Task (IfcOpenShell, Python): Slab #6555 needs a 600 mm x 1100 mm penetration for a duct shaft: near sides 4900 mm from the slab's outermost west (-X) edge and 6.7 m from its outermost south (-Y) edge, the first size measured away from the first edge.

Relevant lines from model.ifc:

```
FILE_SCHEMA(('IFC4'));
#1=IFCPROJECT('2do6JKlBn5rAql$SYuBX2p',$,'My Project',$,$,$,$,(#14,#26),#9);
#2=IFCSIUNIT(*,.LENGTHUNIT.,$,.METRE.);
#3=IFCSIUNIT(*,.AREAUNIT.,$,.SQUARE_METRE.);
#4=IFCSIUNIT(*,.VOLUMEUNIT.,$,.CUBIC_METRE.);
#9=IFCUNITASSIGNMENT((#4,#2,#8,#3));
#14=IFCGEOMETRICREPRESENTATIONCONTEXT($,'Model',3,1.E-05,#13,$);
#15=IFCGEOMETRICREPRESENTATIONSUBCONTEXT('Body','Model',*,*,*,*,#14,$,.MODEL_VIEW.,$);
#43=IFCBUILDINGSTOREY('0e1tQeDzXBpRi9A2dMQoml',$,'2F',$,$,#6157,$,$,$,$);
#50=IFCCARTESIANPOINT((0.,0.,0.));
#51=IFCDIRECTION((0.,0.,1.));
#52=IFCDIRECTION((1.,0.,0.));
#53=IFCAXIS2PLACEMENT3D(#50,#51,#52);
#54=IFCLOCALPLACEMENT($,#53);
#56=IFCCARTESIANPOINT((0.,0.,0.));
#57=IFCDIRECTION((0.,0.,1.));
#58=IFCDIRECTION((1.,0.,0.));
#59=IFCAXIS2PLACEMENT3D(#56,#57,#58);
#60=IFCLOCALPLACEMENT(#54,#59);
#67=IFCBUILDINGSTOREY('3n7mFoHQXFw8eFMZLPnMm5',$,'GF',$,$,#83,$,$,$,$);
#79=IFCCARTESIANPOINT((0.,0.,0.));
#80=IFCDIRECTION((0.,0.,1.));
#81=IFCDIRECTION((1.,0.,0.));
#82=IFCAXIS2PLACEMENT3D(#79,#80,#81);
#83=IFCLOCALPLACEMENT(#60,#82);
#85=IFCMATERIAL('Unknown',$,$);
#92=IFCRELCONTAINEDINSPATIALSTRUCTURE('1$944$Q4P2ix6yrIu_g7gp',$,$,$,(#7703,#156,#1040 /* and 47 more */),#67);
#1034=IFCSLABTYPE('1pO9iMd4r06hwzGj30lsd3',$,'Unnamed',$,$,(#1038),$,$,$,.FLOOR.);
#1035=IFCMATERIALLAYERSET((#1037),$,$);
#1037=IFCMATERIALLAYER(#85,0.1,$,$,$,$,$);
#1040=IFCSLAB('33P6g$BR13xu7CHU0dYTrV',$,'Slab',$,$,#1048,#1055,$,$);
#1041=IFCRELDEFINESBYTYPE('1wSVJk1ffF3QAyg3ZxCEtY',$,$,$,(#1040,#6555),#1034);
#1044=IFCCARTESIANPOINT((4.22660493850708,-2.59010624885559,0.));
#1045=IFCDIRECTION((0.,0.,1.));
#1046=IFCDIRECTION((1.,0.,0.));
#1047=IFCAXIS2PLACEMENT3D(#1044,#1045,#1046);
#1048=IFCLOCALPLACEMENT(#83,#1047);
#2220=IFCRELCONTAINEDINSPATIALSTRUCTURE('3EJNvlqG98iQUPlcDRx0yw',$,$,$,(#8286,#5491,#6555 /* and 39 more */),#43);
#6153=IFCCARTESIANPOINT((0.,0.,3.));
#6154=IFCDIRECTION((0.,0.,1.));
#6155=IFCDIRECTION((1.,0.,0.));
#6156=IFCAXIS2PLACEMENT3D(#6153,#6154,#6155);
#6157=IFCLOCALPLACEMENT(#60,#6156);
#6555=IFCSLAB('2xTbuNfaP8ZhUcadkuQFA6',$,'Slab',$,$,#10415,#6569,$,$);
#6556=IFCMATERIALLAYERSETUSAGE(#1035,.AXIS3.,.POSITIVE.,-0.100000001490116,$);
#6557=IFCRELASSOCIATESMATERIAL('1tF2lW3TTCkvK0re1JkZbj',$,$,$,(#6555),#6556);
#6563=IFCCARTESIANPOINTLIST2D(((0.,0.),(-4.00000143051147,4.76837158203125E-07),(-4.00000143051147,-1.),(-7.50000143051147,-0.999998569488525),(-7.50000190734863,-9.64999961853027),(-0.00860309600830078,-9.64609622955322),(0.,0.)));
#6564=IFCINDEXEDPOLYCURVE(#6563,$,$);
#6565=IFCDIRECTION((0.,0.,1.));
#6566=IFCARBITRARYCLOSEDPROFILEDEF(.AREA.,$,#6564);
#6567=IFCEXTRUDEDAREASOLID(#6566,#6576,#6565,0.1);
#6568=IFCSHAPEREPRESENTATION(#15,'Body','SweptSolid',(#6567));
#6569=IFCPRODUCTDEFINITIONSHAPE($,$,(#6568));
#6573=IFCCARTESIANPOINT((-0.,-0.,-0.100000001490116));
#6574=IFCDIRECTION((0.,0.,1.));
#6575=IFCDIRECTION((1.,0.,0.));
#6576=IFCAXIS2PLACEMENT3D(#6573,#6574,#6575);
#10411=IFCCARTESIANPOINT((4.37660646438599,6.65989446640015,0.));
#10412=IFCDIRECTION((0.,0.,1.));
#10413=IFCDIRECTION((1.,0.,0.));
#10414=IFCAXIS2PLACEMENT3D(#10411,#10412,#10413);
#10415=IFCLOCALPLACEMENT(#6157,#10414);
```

```python
import numpy as np
import ifcopenshell
import ifcopenshell.api.feature
import ifcopenshell.api.geometry
import ifcopenshell.api.root
import ifcopenshell.geom
import ifcopenshell.util.placement
import ifcopenshell.util.representation
import ifcopenshell.util.shape
import ifcopenshell.util.unit

model = ifcopenshell.open("model.ifc")
unit_scale = ifcopenshell.util.unit.calculate_unit_scale(model)
settings = ifcopenshell.geom.settings()


def volume(element):
    """Net volume in cubic metres, openings subtracted."""
    shape = ifcopenshell.geom.create_shape(settings, element)
    return ifcopenshell.util.shape.get_volume(shape.geometry)


slab = model.by_id(6555)
before = volume(slab)

# Extent in the slab's own axes, in metres. The edges named are its -X and -Y sides.
slab_shape = ifcopenshell.geom.create_shape(settings, slab)
vertices = ifcopenshell.util.shape.get_vertices(slab_shape.geometry)
x_min, y_min, bottom = vertices.min(axis=0)
top = vertices[:, 2].max()

opening = ifcopenshell.api.root.create_entity(model, ifc_class="IfcOpeningElement", name="Duct shaft opening", predefined_type="OPENING")
context = ifcopenshell.util.representation.get_context(model, "Model", "Body", "MODEL_VIEW")
width, depth = 0.6, 1.1
outline = [(0.0, 0.0), (width, 0.0), (width, depth), (0.0, depth), (0.0, 0.0)]
# Overshoot both faces by 50 mm so the cut is clean.
shape = ifcopenshell.api.geometry.add_slab_representation(
    model, context=context, depth=top - bottom + 0.1, polyline=outline
)
ifcopenshell.api.geometry.assign_representation(model, product=opening, representation=shape)

matrix = ifcopenshell.util.placement.get_local_placement(slab.ObjectPlacement)
matrix[:, 3] = matrix @ np.append(np.array([x_min + 4.9, y_min + 6.7, bottom - 0.05]) / unit_scale, 1.0)
ifcopenshell.api.geometry.edit_object_placement(model, product=opening, matrix=matrix, is_si=False)
ifcopenshell.api.feature.add_feature(model, feature=opening, element=slab)

after = volume(slab)

print(f"slab volume {before:.3f} -> {after:.3f} m3")

model.write("model-out.ifc")
```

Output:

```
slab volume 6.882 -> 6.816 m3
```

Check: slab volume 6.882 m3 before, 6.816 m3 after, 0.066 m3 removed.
